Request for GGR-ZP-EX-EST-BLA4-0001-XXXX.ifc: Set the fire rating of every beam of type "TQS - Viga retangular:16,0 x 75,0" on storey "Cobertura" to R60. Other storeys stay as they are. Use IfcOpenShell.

First a look at what the model holds.

```python
import ifcopenshell
import ifcopenshell.util.element

model = ifcopenshell.open("GGR-ZP-EX-EST-BLA4-0001-XXXX.ifc")
print(model.schema)
storey = next(s for s in model.by_type("IfcBuildingStorey") if s.Name == "Cobertura")
beams = [e for e in ifcopenshell.util.element.get_decomposition(storey) if e.is_a("IfcBeam")]
seen = {}
for e in beams:
    element_type = ifcopenshell.util.element.get_type(e)
    key = (element_type.Name if element_type != e and element_type else None, ifcopenshell.util.element.get_pset(e, "Pset_BeamCommon", "FireRating"))
    seen[key] = seen.get(key, 0) + 1
for (name, value), count in sorted(seen.items(), key=str):
    print(count, "x", name, "|", value)
```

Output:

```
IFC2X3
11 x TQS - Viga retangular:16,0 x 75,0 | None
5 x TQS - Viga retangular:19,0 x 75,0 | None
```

```python
import ifcopenshell
import ifcopenshell.api.pset
import ifcopenshell.util.element

model = ifcopenshell.open("GGR-ZP-EX-EST-BLA4-0001-XXXX.ifc")

storey = next(s for s in model.by_type("IfcBuildingStorey") if s.Name == "Cobertura")
beams = [e for e in ifcopenshell.util.element.get_decomposition(storey) if e.is_a("IfcBeam")]

count = 0
for e in beams:
    element_type = ifcopenshell.util.element.get_type(e)
    if element_type in (None, e) or element_type.Name != "TQS - Viga retangular:16,0 x 75,0":
        continue
    # add_pset returns the element's existing set when there is one.
    pset = ifcopenshell.api.pset.add_pset(model, product=e, name="Pset_BeamCommon")
    ifcopenshell.api.pset.edit_pset(model, pset=pset, properties={"FireRating": "R60"})
    count += 1

print(count, "beams updated")

model.write("GGR-ZP-EX-EST-BLA4-0001-XXXX_v2.ifc")
```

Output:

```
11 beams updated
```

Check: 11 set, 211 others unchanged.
